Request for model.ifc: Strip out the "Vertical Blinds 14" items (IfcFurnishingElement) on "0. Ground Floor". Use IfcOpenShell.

First a look at what the model holds.

```python
import ifcopenshell
import ifcopenshell.util.element

model = ifcopenshell.open("model.ifc")
print(model.schema)
storey = next(s for s in model.by_type("IfcBuildingStorey") if s.Name == "0. Ground Floor")
furniture = [e for e in ifcopenshell.util.element.get_decomposition(storey) if e.is_a("IfcFurnishingElement")]
seen = {}
for e in furniture:
    element_type = ifcopenshell.util.element.get_type(e)
    name = element_type.Name if element_type not in (None, e) else None
    seen[name] = seen.get(name, 0) + 1
for name, count in sorted(seen.items(), key=str):
    print(count, "x", name)
```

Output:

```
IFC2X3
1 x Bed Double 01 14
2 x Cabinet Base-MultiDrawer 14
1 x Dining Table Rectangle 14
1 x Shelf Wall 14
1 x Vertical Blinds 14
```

```python
import ifcopenshell
import ifcopenshell.api.root
import ifcopenshell.util.element

model = ifcopenshell.open("model.ifc")

storey = next(s for s in model.by_type("IfcBuildingStorey") if s.Name == "0. Ground Floor")
furniture = [e for e in ifcopenshell.util.element.get_decomposition(storey) if e.is_a("IfcFurnishingElement")]
targets = [e for e in furniture if (t := ifcopenshell.util.element.get_type(e)) not in (None, e) and t.Name == "Vertical Blinds 14"]

for e in targets:
    ifcopenshell.api.root.remove_product(model, product=e)
print(len(targets), "removed")

model.write("model_rev.ifc")
```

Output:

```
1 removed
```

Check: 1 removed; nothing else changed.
